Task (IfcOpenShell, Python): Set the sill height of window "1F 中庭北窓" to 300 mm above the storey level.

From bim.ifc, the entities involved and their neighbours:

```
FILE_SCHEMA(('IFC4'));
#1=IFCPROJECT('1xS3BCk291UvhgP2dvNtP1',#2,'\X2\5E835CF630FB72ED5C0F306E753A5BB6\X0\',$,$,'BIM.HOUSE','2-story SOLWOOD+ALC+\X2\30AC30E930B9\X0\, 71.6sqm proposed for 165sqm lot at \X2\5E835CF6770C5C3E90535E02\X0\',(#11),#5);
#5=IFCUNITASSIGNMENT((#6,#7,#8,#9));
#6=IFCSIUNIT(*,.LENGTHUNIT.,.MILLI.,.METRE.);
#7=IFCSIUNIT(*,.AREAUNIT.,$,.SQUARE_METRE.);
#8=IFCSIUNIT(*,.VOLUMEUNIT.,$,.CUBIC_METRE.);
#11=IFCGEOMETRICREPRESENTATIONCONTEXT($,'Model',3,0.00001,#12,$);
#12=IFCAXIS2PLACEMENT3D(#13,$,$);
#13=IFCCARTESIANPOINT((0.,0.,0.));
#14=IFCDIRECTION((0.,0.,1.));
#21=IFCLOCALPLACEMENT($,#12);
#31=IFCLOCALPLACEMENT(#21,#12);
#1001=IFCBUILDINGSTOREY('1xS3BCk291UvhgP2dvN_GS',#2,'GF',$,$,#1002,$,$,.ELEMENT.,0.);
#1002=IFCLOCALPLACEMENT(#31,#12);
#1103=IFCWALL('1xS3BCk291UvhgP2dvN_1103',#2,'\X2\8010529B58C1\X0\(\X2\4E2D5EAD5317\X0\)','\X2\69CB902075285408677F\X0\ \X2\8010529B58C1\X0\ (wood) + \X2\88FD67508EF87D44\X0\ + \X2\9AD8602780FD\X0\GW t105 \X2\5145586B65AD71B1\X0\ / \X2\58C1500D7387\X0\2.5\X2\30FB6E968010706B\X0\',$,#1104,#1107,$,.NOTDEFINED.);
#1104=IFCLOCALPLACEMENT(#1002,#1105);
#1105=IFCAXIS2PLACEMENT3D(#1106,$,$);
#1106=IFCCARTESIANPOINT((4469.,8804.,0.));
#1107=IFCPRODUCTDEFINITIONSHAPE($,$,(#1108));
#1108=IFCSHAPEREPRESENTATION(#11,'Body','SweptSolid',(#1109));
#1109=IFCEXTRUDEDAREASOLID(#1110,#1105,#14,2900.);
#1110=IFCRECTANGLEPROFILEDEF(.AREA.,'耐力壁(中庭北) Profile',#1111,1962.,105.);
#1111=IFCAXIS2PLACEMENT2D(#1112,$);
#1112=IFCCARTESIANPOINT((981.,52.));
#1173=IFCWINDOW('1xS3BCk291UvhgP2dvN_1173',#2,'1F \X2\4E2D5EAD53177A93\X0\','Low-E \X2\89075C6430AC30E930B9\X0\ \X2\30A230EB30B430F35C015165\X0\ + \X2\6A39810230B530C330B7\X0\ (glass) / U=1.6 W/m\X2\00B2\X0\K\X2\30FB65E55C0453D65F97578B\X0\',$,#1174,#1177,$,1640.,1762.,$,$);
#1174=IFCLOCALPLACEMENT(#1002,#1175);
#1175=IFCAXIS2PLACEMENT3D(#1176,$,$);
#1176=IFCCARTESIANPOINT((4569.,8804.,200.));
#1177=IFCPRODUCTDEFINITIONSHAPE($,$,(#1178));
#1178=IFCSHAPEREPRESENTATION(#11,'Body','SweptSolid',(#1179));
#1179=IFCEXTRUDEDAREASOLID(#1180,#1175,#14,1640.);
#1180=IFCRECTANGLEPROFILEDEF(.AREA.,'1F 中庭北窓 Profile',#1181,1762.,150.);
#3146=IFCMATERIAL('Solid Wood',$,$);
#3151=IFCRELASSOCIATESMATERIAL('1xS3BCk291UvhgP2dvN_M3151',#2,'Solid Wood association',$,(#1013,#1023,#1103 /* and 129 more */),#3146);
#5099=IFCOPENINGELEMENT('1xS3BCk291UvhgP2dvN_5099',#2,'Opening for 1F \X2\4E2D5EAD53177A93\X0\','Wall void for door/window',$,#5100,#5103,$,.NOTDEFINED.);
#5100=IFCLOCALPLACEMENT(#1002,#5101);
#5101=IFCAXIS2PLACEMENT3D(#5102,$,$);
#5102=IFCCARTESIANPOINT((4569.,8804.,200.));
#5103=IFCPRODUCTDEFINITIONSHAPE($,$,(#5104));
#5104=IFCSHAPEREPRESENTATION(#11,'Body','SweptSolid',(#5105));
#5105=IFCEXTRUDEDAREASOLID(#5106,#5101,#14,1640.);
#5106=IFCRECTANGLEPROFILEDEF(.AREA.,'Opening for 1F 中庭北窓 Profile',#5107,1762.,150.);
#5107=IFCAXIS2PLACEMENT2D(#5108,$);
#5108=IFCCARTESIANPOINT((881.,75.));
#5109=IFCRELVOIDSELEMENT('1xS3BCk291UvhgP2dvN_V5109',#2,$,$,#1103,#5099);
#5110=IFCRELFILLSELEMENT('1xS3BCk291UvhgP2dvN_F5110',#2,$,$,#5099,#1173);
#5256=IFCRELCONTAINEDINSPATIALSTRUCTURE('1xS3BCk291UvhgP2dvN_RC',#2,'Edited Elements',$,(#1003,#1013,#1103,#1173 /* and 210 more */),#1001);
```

```python
import numpy as np
import ifcopenshell
import ifcopenshell.api.geometry
import ifcopenshell.geom
import ifcopenshell.util.element
import ifcopenshell.util.placement
import ifcopenshell.util.shape
import ifcopenshell.util.unit

model = ifcopenshell.open("bim.ifc")
unit_scale = ifcopenshell.util.unit.calculate_unit_scale(model)

window = model.by_id(1173)
opening = window.FillsVoids[0].RelatingOpeningElement
storey = ifcopenshell.util.element.get_container(window, ifc_class="IfcBuildingStorey")
level = ifcopenshell.util.placement.get_local_placement(storey.ObjectPlacement)[2, 3]

# The opening's origin need not be at the sill, so measure its lowest point.
shape = ifcopenshell.geom.create_shape(ifcopenshell.geom.settings(), opening)
bottom = ifcopenshell.util.shape.get_shape_bottom_elevation(shape, shape.geometry) / unit_scale
dz = level + 300.0 - bottom

shift = np.array([0.0, 0.0, dz])
# The window is not placed relative to its opening, so move both.
for product in (opening, window):
    matrix = ifcopenshell.util.placement.get_local_placement(product.ObjectPlacement)
    matrix[:3, 3] += shift
    ifcopenshell.api.geometry.edit_object_placement(model, product=product, matrix=matrix, is_si=False)

print(f"moved by {dz * unit_scale:+.3f} m")

model.write("bim_updated.ifc")
```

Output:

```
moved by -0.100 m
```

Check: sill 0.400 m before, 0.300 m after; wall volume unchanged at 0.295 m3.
